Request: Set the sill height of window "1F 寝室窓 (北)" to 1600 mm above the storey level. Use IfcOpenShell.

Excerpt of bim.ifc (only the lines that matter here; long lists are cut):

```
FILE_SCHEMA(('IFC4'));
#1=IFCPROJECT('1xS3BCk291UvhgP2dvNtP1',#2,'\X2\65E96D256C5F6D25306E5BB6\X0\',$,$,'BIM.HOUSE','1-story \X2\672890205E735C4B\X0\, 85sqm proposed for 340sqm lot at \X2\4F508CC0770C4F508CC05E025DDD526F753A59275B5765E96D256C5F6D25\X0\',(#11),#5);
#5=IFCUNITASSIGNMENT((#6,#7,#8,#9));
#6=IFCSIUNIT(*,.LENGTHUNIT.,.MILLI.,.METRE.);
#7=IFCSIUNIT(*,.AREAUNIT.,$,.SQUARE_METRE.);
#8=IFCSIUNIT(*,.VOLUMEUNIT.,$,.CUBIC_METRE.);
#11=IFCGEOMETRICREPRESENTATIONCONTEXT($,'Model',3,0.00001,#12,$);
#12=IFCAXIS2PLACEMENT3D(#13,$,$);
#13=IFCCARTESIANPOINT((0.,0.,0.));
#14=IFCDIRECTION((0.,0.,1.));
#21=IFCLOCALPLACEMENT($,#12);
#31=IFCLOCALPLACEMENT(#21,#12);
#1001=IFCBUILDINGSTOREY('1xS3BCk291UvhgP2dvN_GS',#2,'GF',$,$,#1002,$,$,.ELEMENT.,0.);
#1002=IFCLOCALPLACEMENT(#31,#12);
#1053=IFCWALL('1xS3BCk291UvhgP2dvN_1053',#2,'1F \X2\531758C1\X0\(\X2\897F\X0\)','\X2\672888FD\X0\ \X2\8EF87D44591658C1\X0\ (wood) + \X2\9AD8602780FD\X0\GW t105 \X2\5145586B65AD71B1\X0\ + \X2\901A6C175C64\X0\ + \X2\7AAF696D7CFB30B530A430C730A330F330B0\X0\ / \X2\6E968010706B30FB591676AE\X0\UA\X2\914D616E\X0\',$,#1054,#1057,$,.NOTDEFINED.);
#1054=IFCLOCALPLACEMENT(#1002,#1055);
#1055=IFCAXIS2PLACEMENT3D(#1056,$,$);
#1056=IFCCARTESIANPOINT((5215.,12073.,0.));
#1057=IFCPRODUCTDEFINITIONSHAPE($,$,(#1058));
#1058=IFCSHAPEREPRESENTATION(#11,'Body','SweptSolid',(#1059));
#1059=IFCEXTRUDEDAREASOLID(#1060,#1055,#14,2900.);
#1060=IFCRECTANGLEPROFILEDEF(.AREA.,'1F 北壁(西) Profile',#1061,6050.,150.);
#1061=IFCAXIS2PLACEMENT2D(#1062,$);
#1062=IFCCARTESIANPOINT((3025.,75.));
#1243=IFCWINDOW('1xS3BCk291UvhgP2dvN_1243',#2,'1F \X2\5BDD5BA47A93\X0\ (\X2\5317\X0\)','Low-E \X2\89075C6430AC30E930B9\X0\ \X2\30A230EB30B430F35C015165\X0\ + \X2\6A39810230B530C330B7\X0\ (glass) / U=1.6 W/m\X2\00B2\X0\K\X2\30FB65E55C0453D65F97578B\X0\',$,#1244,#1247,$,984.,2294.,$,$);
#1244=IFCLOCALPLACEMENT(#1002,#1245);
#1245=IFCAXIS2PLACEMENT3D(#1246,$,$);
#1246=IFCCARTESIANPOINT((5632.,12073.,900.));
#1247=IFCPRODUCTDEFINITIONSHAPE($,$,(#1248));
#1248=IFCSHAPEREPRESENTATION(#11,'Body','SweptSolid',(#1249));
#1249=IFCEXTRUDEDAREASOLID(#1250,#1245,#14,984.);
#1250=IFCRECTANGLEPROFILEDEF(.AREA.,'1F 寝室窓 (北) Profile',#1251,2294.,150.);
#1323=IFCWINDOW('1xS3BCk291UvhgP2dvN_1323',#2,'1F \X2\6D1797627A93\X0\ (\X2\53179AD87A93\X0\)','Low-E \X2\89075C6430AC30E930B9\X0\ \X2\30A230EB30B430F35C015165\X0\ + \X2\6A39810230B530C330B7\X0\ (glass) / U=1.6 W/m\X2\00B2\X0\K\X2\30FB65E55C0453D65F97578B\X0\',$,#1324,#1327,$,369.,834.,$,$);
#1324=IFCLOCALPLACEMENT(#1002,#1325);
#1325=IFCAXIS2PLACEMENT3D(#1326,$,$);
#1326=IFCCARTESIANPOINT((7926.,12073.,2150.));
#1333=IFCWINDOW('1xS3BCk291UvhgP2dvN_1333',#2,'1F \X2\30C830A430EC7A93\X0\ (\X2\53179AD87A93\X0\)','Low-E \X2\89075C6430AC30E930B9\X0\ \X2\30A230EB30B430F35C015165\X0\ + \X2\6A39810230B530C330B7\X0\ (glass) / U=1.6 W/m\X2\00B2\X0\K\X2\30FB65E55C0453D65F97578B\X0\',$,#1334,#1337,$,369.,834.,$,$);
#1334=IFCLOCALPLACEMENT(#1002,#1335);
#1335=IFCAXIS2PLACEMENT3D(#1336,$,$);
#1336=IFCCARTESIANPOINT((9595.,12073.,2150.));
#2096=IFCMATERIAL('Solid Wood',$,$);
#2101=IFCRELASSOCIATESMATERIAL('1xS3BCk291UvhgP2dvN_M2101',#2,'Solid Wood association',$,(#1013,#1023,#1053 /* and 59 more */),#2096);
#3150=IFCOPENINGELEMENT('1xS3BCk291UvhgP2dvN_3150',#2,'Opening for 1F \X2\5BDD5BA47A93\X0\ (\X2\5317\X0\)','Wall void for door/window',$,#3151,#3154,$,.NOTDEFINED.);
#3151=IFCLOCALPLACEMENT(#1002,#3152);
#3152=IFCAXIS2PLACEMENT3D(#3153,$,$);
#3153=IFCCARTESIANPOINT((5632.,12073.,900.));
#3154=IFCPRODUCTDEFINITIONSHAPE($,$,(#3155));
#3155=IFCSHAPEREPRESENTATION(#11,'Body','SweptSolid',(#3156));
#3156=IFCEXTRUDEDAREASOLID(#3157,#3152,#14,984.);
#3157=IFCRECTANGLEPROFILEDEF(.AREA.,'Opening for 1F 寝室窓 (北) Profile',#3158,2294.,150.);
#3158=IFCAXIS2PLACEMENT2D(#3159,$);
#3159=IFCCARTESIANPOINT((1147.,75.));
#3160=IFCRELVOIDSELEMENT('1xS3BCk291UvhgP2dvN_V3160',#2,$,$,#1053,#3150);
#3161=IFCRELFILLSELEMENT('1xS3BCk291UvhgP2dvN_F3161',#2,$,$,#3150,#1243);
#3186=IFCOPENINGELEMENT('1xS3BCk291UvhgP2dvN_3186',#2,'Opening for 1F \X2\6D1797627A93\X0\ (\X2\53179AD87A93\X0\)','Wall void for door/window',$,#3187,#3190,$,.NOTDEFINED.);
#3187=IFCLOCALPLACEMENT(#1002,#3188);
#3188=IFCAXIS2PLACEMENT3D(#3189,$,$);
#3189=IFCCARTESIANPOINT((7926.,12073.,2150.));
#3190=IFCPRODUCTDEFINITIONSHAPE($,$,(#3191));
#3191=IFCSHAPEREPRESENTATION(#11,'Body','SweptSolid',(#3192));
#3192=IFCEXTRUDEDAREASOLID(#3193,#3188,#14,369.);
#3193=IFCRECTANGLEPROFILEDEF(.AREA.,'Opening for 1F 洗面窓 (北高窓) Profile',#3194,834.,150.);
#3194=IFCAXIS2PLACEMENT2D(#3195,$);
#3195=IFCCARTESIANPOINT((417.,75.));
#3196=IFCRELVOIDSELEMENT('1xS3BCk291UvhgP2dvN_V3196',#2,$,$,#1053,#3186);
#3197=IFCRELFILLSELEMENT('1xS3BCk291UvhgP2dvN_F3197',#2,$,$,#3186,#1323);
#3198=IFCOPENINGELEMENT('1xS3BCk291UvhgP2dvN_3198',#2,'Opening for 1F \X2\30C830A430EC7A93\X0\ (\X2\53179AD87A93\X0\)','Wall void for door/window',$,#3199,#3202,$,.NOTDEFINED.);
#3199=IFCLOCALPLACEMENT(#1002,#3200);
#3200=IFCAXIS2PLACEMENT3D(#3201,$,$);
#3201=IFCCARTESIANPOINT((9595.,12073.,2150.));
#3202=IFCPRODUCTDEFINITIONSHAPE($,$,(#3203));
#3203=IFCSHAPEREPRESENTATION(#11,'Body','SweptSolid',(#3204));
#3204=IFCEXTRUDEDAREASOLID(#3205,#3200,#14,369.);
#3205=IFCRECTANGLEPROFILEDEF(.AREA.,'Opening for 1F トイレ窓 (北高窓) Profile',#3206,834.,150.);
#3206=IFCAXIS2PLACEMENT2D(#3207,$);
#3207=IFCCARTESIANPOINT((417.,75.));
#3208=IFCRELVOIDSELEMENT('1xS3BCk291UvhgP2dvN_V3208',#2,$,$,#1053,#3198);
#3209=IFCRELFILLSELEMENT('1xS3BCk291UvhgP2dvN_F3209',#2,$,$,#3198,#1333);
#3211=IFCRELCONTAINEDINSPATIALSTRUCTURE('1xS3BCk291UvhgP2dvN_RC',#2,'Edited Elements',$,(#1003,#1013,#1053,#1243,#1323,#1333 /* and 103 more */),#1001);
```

```python
import numpy as np
import ifcopenshell
import ifcopenshell.api.geometry
import ifcopenshell.geom
import ifcopenshell.util.element
import ifcopenshell.util.placement
import ifcopenshell.util.shape
import ifcopenshell.util.unit

model = ifcopenshell.open("bim.ifc")
unit_scale = ifcopenshell.util.unit.calculate_unit_scale(model)

window = model.by_guid("1xS3BCk291UvhgP2dvN_1243")
opening = window.FillsVoids[0].RelatingOpeningElement
storey = ifcopenshell.util.element.get_container(window, ifc_class="IfcBuildingStorey")
level = ifcopenshell.util.placement.get_local_placement(storey.ObjectPlacement)[2, 3]

# The opening's origin need not be at the sill, so measure its lowest point.
shape = ifcopenshell.geom.create_shape(ifcopenshell.geom.settings(), opening)
bottom = ifcopenshell.util.shape.get_shape_bottom_elevation(shape, shape.geometry) / unit_scale
dz = level + 1.6 / unit_scale - bottom

shift = np.array([0.0, 0.0, dz])
# The window is not placed relative to its opening, so move both.
for product in (opening, window):
    matrix = ifcopenshell.util.placement.get_local_placement(product.ObjectPlacement)
    matrix[:3, 3] += shift
    ifcopenshell.api.geometry.edit_object_placement(model, product=product, matrix=matrix, is_si=False)

print(f"moved by {dz * unit_scale:+.3f} m")

model.write("bim_edited.ifc")
```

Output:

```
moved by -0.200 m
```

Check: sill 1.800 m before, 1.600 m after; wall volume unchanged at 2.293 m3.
